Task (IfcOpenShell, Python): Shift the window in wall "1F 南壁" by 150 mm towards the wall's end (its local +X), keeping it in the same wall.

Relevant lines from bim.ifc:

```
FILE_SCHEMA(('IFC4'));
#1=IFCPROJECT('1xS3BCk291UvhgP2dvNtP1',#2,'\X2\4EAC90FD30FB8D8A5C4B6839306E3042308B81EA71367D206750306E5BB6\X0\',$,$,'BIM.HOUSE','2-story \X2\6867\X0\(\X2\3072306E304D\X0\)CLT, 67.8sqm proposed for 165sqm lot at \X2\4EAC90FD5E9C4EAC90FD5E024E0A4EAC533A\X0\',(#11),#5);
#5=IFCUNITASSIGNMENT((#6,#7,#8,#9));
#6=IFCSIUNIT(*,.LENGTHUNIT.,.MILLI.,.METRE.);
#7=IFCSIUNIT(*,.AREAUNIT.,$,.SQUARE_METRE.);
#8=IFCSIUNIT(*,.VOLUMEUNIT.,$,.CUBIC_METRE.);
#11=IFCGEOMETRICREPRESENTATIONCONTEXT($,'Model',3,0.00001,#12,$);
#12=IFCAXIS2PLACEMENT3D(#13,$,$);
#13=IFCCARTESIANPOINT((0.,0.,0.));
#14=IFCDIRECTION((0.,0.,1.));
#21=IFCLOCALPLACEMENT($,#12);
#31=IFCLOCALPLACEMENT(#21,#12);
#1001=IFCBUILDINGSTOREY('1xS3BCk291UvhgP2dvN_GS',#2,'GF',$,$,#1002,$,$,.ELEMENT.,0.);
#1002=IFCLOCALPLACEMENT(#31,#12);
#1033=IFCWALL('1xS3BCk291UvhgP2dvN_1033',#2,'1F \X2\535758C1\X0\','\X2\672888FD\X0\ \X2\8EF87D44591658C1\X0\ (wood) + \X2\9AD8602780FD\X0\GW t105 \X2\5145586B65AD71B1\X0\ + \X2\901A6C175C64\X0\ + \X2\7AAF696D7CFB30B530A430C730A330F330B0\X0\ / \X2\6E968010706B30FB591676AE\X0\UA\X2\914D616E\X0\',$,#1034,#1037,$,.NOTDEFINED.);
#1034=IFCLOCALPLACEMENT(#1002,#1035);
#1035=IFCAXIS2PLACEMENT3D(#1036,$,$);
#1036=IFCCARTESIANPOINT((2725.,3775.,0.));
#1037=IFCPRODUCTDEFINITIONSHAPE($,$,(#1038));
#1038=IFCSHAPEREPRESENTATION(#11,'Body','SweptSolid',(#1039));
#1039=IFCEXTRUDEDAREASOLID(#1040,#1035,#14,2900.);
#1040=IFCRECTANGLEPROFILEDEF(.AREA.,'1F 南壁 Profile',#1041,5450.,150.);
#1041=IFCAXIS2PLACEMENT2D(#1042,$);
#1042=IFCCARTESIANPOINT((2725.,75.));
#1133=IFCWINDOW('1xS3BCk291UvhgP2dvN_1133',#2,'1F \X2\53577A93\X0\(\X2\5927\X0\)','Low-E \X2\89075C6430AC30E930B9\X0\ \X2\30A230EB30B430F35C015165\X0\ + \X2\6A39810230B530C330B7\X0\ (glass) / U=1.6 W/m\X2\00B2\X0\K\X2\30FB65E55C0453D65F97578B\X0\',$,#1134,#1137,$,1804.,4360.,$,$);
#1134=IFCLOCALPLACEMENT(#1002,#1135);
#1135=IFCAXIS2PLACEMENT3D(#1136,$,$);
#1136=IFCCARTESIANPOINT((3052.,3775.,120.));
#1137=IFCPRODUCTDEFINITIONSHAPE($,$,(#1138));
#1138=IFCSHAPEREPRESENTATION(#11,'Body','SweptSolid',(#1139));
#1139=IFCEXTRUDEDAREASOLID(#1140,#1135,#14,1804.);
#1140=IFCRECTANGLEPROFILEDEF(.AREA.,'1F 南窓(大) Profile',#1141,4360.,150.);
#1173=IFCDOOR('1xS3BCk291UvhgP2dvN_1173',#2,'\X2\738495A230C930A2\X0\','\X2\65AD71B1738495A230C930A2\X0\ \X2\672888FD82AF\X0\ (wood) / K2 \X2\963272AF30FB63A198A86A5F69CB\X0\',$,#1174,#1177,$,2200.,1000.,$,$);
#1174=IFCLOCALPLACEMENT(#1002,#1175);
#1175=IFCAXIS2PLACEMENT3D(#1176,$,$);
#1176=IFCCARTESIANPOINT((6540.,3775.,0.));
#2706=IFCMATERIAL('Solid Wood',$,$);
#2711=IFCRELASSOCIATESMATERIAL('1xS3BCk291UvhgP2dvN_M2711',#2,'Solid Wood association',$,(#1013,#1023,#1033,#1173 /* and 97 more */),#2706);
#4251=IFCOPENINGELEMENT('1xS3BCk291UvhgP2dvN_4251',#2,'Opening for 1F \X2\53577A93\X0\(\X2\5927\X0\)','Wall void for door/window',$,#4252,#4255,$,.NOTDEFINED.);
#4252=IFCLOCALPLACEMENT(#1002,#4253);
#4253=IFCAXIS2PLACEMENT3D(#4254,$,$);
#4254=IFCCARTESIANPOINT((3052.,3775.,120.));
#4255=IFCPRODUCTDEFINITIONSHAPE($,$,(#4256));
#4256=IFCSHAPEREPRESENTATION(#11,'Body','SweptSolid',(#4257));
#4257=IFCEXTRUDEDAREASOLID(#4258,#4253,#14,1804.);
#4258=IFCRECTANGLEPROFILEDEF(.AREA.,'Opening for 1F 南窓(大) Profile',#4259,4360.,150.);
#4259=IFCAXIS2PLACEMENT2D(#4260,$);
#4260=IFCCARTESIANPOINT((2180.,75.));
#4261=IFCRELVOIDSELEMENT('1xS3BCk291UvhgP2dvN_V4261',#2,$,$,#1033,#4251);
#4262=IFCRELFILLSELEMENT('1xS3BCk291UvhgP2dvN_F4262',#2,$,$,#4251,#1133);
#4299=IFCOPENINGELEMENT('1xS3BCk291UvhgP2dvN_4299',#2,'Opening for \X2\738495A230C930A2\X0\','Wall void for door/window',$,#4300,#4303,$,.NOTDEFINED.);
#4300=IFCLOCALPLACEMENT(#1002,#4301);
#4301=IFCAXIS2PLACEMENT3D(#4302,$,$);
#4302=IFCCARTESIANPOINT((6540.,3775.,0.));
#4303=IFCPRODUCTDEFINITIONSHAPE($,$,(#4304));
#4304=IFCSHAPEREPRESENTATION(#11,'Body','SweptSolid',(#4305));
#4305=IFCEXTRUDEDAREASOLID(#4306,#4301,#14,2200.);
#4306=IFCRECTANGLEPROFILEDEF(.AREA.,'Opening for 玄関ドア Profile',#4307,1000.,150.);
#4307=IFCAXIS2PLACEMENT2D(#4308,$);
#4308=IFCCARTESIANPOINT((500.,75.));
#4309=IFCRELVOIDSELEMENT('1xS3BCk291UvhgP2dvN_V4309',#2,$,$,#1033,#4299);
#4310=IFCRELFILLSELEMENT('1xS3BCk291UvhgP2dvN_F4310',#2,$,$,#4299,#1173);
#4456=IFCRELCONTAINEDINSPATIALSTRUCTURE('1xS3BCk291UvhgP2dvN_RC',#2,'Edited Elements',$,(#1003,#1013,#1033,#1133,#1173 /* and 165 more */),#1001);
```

```python
import ifcopenshell
import ifcopenshell.api.geometry
import ifcopenshell.util.placement
import ifcopenshell.util.unit

model = ifcopenshell.open("bim.ifc")
unit_scale = ifcopenshell.util.unit.calculate_unit_scale(model)

window = model.by_guid("1xS3BCk291UvhgP2dvN_1133")
opening = window.FillsVoids[0].RelatingOpeningElement
wall = opening.VoidsElements[0].RelatingBuildingElement

wall_matrix = ifcopenshell.util.placement.get_local_placement(wall.ObjectPlacement)
shift = wall_matrix[:3, 0] * 0.15 / unit_scale
before = ifcopenshell.util.placement.get_local_placement(window.ObjectPlacement)[:3, 3].copy()

# The window is not placed relative to its opening, so move both.
for product in (opening, window):
    matrix = ifcopenshell.util.placement.get_local_placement(product.ObjectPlacement)
    matrix[:3, 3] += shift
    ifcopenshell.api.geometry.edit_object_placement(model, product=product, matrix=matrix, is_si=False)

after = ifcopenshell.util.placement.get_local_placement(window.ObjectPlacement)[:3, 3]
print("window moved by", (after - before).round(3) + 0.0)

model.write("bim-out.ifc")
```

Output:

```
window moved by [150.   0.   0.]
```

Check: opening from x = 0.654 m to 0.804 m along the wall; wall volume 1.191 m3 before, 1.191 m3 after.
